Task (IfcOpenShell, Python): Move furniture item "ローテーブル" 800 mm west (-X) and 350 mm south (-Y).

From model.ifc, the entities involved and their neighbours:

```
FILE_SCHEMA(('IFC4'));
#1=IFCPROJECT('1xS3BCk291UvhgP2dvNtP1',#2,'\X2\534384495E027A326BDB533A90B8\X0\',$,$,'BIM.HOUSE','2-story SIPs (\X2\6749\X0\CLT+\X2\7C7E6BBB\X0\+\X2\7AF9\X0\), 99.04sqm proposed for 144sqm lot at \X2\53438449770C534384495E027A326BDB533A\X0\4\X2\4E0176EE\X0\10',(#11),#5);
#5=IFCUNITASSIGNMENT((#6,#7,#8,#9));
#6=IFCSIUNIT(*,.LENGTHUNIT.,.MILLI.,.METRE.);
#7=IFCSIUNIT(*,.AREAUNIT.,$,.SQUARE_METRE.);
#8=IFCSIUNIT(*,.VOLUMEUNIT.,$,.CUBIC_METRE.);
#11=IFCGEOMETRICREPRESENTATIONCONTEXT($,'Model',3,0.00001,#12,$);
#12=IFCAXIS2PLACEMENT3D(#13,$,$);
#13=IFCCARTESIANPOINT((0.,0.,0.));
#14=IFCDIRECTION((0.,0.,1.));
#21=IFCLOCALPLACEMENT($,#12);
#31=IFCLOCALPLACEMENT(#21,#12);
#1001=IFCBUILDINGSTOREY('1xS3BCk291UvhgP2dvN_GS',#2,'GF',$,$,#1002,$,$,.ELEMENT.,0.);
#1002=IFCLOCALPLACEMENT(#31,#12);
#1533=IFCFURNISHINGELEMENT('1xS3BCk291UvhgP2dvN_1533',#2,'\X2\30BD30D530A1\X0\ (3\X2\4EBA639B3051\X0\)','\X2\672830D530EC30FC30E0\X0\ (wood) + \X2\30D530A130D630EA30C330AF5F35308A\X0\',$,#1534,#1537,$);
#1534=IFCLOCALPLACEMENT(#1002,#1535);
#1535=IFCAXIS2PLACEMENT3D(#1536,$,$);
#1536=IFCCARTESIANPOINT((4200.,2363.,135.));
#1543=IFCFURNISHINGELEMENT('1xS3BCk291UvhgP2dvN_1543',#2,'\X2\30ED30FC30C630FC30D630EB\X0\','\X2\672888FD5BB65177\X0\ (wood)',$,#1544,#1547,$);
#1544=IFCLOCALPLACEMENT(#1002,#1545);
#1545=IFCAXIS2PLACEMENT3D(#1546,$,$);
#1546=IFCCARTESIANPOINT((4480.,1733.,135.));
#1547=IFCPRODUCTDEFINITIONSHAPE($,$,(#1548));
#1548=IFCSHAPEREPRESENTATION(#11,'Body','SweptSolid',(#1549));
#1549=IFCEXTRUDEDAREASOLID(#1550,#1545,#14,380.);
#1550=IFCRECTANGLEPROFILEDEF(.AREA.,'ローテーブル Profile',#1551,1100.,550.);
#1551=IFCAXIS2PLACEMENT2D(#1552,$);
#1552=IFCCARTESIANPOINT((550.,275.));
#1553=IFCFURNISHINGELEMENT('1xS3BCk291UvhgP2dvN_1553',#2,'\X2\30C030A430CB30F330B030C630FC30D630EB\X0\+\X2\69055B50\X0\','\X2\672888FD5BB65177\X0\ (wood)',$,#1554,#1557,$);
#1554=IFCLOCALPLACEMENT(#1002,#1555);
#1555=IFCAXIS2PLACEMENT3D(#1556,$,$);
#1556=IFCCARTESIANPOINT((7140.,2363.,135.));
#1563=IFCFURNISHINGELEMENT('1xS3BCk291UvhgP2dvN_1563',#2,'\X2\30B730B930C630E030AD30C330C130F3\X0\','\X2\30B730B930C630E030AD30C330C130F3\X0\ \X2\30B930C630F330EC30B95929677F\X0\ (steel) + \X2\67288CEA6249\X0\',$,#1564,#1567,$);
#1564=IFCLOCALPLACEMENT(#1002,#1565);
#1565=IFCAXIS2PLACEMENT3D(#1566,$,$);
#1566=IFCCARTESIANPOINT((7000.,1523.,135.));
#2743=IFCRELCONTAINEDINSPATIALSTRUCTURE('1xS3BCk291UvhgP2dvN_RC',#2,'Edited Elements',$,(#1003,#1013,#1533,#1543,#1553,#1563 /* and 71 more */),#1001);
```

```python
import ifcopenshell
import ifcopenshell.api.geometry
import ifcopenshell.util.placement
import ifcopenshell.util.unit

model = ifcopenshell.open("model.ifc")
unit_scale = ifcopenshell.util.unit.calculate_unit_scale(model)

item = model.by_id(1543)
matrix = ifcopenshell.util.placement.get_local_placement(item.ObjectPlacement)
matrix[0, 3] -= 0.8 / unit_scale
matrix[1, 3] -= 0.35 / unit_scale
ifcopenshell.api.geometry.edit_object_placement(model, product=item, matrix=matrix, is_si=False)

print(ifcopenshell.util.placement.get_local_placement(item.ObjectPlacement).round(3) + 0.0)

model.write("model_v2.ifc")
```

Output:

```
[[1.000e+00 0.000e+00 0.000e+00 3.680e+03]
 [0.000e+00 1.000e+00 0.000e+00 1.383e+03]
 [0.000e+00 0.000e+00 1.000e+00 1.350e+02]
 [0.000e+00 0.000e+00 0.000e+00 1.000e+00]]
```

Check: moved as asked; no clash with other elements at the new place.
